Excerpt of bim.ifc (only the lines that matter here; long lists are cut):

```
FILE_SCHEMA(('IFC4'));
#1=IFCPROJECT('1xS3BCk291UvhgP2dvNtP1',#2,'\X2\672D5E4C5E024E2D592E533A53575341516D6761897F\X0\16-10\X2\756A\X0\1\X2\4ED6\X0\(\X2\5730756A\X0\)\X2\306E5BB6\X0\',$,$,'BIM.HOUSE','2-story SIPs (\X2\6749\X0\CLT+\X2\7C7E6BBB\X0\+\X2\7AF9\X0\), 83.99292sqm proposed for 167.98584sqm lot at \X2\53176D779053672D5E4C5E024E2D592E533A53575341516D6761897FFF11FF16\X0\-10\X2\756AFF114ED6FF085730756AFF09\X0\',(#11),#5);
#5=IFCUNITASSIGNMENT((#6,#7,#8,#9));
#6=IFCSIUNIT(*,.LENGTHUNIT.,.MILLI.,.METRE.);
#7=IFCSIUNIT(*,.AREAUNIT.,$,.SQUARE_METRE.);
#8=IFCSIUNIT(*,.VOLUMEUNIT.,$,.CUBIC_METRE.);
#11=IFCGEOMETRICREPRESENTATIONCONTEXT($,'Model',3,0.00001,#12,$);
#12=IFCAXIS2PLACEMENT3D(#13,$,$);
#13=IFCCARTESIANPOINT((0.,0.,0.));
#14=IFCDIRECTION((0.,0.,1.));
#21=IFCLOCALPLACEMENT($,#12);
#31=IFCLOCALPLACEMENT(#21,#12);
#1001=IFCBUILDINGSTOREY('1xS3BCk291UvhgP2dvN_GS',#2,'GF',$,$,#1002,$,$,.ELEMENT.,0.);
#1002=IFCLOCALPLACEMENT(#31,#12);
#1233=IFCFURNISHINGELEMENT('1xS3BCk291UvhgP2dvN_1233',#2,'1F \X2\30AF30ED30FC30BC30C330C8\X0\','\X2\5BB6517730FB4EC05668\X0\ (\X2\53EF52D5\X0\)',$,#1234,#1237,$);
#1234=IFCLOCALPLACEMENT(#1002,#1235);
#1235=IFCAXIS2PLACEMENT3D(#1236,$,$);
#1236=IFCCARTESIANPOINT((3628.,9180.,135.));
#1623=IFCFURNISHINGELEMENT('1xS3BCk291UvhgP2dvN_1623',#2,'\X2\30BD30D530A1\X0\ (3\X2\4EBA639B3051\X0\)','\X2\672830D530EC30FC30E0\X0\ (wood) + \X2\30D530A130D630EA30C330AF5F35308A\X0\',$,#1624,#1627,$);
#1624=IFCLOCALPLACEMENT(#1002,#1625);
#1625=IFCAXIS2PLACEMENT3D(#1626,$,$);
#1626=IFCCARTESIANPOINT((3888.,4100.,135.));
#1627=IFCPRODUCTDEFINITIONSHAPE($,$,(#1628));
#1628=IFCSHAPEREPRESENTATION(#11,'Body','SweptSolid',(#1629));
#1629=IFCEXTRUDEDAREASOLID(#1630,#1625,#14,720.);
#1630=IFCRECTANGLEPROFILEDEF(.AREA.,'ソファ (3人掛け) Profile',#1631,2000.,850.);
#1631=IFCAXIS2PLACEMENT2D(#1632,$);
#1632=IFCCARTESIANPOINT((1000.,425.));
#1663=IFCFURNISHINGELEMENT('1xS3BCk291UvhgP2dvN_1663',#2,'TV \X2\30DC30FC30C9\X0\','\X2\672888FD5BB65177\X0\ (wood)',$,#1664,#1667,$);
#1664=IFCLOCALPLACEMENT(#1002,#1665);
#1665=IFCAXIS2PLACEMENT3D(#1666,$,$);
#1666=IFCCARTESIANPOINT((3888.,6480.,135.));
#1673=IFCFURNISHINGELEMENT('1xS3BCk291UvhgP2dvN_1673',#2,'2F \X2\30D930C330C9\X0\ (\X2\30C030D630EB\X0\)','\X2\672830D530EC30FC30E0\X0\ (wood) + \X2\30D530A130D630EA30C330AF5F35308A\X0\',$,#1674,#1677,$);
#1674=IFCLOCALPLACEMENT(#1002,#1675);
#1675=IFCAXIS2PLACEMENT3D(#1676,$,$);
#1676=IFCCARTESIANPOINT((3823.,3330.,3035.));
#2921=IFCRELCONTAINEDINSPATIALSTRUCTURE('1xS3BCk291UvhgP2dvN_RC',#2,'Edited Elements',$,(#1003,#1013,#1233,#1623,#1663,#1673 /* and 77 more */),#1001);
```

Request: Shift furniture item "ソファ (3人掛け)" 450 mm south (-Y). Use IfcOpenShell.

```python
import ifcopenshell
import ifcopenshell.api.geometry
import ifcopenshell.util.placement
import ifcopenshell.util.unit

model = ifcopenshell.open("bim.ifc")
unit_scale = ifcopenshell.util.unit.calculate_unit_scale(model)

item = model.by_guid("1xS3BCk291UvhgP2dvN_1623")
matrix = ifcopenshell.util.placement.get_local_placement(item.ObjectPlacement)
matrix[1, 3] -= 0.45 / unit_scale
ifcopenshell.api.geometry.edit_object_placement(model, product=item, matrix=matrix, is_si=False)

print(ifcopenshell.util.placement.get_local_placement(item.ObjectPlacement).round(3) + 0.0)

model.write("bim_edited.ifc")
```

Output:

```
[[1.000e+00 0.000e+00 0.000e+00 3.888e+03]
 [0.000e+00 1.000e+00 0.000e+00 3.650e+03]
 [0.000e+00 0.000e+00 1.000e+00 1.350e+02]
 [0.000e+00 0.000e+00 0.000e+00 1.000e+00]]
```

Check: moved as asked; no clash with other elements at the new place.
